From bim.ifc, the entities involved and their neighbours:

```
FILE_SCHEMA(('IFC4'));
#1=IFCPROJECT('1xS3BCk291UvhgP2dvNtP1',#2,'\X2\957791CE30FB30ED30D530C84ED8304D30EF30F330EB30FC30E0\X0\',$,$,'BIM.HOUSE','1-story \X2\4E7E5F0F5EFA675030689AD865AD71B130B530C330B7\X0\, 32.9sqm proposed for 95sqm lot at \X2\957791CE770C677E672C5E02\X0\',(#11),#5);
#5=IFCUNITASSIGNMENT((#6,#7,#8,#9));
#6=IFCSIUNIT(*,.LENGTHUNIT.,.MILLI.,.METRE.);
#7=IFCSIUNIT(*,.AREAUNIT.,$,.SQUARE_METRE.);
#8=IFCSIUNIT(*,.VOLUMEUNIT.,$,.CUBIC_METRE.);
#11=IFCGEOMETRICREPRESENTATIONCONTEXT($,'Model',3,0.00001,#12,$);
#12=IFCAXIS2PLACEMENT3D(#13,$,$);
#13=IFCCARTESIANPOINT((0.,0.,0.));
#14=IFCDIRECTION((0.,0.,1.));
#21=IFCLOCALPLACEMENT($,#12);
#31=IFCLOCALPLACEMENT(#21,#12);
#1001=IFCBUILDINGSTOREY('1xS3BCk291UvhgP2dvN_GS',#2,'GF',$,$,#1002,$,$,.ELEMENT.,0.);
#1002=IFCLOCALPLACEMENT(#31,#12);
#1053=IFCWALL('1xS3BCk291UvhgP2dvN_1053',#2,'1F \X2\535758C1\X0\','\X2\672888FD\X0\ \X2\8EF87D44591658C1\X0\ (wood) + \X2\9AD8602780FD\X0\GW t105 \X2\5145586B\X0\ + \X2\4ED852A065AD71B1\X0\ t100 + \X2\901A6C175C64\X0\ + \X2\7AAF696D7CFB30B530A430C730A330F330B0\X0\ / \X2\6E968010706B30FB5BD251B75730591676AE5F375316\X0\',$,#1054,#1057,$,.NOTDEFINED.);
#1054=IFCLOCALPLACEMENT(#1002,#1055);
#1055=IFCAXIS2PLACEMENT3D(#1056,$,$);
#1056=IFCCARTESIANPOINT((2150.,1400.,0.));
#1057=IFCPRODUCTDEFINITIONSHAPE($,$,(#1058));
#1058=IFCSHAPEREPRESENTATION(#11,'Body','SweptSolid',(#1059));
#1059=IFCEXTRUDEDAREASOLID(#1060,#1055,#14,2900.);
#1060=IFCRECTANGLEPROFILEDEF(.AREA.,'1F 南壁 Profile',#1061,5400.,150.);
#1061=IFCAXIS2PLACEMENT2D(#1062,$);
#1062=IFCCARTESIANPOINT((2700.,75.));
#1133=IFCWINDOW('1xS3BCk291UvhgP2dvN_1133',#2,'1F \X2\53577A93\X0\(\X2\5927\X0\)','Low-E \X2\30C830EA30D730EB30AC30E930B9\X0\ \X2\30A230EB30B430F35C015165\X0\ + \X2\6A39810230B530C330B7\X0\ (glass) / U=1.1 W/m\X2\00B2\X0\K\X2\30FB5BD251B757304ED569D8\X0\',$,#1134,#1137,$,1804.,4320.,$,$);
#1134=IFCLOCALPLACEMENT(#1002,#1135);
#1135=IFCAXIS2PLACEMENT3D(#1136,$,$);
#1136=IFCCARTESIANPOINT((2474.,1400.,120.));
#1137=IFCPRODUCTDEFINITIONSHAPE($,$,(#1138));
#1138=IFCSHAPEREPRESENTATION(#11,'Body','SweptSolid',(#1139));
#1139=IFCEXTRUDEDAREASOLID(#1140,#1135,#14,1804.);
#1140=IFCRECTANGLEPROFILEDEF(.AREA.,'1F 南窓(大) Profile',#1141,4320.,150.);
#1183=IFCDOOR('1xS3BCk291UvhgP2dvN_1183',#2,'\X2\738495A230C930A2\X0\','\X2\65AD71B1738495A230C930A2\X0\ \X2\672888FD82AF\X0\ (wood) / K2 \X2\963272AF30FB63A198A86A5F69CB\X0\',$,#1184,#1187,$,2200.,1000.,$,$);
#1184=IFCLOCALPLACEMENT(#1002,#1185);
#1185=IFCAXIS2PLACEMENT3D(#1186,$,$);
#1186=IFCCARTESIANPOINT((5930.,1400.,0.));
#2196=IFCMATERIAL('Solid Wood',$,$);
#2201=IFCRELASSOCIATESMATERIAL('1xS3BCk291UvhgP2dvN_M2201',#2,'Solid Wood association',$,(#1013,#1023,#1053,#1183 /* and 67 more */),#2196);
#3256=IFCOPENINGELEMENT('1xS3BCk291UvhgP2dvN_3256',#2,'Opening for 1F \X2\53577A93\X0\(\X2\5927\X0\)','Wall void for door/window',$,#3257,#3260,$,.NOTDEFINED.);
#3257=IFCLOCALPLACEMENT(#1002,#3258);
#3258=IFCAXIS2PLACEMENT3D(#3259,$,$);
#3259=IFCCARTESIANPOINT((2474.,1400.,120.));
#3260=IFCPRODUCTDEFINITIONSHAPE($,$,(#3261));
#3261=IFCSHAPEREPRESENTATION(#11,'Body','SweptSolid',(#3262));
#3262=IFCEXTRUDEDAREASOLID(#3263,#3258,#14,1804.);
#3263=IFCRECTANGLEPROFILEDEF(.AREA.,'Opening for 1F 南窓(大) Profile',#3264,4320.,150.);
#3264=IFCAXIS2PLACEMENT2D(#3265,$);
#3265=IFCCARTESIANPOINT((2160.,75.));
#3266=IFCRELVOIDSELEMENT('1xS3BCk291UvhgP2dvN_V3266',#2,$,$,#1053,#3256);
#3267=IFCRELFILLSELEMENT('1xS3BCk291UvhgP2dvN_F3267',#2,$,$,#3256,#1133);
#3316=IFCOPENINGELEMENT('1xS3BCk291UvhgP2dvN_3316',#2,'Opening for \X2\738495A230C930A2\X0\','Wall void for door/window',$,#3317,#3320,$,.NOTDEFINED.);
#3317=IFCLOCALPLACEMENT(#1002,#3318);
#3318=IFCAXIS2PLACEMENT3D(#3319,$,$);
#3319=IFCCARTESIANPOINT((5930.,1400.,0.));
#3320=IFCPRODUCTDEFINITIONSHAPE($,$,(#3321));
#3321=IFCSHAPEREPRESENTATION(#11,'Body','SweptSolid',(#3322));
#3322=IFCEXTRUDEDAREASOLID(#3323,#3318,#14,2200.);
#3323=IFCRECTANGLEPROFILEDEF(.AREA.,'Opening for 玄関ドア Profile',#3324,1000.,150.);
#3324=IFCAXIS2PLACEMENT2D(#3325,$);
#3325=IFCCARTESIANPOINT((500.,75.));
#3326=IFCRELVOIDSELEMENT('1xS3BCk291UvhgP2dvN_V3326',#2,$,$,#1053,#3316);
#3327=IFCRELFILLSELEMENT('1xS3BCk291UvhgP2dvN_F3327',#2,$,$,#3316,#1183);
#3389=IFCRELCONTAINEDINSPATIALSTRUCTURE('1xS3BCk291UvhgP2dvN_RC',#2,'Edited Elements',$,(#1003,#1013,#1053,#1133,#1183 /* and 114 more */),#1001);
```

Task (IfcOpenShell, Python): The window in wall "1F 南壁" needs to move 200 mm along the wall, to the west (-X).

```python
import ifcopenshell
import ifcopenshell.api.geometry
import ifcopenshell.util.placement

model = ifcopenshell.open("bim.ifc")

window = model.by_guid("1xS3BCk291UvhgP2dvN_1133")
opening = window.FillsVoids[0].RelatingOpeningElement
wall = opening.VoidsElements[0].RelatingBuildingElement

wall_matrix = ifcopenshell.util.placement.get_local_placement(wall.ObjectPlacement)
shift = wall_matrix[:3, 0] * -200.0
before = ifcopenshell.util.placement.get_local_placement(window.ObjectPlacement)[:3, 3].copy()

# The window is not placed relative to its opening, so move both.
for product in (opening, window):
    matrix = ifcopenshell.util.placement.get_local_placement(product.ObjectPlacement)
    matrix[:3, 3] += shift
    ifcopenshell.api.geometry.edit_object_placement(model, product=product, matrix=matrix, is_si=False)

after = ifcopenshell.util.placement.get_local_placement(window.ObjectPlacement)[:3, 3]
print("window moved by", (after - before).round(3) + 0.0)

model.write("bim_edited.ifc")
```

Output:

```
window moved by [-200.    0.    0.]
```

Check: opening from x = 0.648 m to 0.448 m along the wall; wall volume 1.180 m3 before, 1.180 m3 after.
